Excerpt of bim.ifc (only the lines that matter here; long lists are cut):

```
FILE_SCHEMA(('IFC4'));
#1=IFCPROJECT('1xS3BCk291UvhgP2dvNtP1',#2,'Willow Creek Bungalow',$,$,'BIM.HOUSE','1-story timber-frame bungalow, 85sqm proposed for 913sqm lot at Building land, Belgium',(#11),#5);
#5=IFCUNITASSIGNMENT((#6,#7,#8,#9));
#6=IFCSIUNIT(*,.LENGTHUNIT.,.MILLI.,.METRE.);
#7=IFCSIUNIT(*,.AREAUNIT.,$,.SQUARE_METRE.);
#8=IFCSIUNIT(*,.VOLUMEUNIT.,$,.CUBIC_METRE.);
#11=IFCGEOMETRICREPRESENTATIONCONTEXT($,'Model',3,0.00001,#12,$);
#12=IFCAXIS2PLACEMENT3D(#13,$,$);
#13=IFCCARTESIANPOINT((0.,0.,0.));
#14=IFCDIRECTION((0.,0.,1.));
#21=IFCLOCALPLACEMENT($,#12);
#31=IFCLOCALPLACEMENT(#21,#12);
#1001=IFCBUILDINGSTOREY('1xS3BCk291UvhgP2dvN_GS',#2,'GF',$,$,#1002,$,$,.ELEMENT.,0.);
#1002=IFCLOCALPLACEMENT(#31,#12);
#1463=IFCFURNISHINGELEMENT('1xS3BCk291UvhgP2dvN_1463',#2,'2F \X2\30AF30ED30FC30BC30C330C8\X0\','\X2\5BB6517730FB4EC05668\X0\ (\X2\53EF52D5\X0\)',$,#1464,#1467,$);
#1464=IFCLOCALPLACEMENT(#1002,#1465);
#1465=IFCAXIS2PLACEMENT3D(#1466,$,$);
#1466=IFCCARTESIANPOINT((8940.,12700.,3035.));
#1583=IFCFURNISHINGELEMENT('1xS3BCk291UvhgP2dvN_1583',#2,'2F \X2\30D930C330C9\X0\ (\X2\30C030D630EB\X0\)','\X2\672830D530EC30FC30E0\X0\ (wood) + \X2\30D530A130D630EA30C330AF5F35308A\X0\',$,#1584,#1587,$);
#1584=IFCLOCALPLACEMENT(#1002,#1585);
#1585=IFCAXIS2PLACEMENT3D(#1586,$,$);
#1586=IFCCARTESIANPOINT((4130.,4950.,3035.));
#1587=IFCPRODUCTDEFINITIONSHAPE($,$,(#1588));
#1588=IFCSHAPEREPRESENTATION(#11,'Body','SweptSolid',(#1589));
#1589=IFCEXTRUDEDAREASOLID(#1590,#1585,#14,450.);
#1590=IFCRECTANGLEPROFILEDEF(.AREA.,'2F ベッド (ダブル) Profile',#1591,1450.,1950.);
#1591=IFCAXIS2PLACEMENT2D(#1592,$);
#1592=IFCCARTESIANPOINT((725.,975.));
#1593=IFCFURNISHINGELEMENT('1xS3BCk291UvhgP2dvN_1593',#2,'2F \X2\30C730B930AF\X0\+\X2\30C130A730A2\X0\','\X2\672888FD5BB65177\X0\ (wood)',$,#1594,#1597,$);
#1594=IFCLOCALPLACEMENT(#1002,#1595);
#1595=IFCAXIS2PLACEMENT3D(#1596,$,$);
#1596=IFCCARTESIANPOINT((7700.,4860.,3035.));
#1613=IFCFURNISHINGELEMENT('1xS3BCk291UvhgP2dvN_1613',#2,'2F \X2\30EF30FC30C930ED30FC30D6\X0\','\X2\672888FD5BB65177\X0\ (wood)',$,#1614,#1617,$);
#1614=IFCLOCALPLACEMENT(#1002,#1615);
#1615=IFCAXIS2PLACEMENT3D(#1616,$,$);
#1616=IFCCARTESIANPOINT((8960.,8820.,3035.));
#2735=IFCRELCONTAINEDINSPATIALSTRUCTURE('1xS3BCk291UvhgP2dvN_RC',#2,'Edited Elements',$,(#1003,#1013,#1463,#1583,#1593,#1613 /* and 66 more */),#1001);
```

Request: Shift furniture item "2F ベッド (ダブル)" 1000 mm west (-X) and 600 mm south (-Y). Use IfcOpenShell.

```python
import ifcopenshell
import ifcopenshell.api.geometry
import ifcopenshell.util.placement

model = ifcopenshell.open("bim.ifc")

item = model.by_id(1583)
matrix = ifcopenshell.util.placement.get_local_placement(item.ObjectPlacement)
matrix[0, 3] -= 1000.0
matrix[1, 3] -= 600.0
ifcopenshell.api.geometry.edit_object_placement(model, product=item, matrix=matrix, is_si=False)

print(ifcopenshell.util.placement.get_local_placement(item.ObjectPlacement).round(3) + 0.0)

model.write("bim_edited.ifc")
```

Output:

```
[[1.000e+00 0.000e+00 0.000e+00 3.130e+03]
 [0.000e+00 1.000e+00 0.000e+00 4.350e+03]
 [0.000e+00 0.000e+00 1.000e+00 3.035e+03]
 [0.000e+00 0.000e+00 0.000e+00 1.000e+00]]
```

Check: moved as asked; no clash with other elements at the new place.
